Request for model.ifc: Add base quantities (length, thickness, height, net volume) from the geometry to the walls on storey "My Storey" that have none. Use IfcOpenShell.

First a look at what the model holds.

```python
import ifcopenshell
import ifcopenshell.util.element
import ifcopenshell.util.unit

model = ifcopenshell.open("model.ifc")
print(model.schema)
for unit_type in ("LENGTHUNIT", "AREAUNIT", "VOLUMEUNIT"):
    print(unit_type, ifcopenshell.util.unit.calculate_unit_scale(model, unit_type))
storey = next(s for s in model.by_type("IfcBuildingStorey") if s.Name == "My Storey")
walls = [e for e in ifcopenshell.util.element.get_decomposition(storey) if e.is_a("IfcWall")]
for e in sorted(walls, key=lambda e: e.id()):
    print(e.id(), e.is_a(), e.Name, list(ifcopenshell.util.element.get_psets(e, qtos_only=True)), sep=" | ")
```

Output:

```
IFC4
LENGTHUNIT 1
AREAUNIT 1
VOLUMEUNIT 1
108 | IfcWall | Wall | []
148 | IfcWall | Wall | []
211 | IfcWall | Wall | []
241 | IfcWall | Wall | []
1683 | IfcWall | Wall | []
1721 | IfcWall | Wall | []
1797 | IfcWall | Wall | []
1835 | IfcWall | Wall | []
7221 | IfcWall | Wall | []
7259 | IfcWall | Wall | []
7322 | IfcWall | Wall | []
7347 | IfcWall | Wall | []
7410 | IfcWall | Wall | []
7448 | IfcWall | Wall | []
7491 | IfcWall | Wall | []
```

```python
import ifcopenshell
import ifcopenshell.api.pset
import ifcopenshell.geom
import ifcopenshell.util.element
import ifcopenshell.util.shape
import ifcopenshell.util.unit

model = ifcopenshell.open("model.ifc")
unit_scale = ifcopenshell.util.unit.calculate_unit_scale(model)
volume_scale = ifcopenshell.util.unit.calculate_unit_scale(model, "VOLUMEUNIT")
settings = ifcopenshell.geom.settings()

storey = next(s for s in model.by_type("IfcBuildingStorey") if s.Name == "My Storey")
walls = [e for e in ifcopenshell.util.element.get_decomposition(storey) if e.is_a("IfcWall")]

for e in sorted(walls, key=lambda e: e.id()):
    if ifcopenshell.util.element.get_psets(e, qtos_only=True, should_inherit=False):
        continue
    # Geometry comes back in metres, in the element's own axes.
    shape = ifcopenshell.geom.create_shape(settings, e)
    values = {
        "Length": ifcopenshell.util.shape.get_x(shape.geometry) / unit_scale,
        "Width": ifcopenshell.util.shape.get_y(shape.geometry) / unit_scale,
        "Height": ifcopenshell.util.shape.get_z(shape.geometry) / unit_scale,
        "NetVolume": ifcopenshell.util.shape.get_volume(shape.geometry) / volume_scale,
    }
    qto = ifcopenshell.api.pset.add_qto(model, product=e, name="Qto_WallBaseQuantities")
    ifcopenshell.api.pset.edit_qto(model, qto=qto, properties=values)
    print(e.id(), {k: round(v, 3) for k, v in values.items()})

model.write("model_v2.ifc")
```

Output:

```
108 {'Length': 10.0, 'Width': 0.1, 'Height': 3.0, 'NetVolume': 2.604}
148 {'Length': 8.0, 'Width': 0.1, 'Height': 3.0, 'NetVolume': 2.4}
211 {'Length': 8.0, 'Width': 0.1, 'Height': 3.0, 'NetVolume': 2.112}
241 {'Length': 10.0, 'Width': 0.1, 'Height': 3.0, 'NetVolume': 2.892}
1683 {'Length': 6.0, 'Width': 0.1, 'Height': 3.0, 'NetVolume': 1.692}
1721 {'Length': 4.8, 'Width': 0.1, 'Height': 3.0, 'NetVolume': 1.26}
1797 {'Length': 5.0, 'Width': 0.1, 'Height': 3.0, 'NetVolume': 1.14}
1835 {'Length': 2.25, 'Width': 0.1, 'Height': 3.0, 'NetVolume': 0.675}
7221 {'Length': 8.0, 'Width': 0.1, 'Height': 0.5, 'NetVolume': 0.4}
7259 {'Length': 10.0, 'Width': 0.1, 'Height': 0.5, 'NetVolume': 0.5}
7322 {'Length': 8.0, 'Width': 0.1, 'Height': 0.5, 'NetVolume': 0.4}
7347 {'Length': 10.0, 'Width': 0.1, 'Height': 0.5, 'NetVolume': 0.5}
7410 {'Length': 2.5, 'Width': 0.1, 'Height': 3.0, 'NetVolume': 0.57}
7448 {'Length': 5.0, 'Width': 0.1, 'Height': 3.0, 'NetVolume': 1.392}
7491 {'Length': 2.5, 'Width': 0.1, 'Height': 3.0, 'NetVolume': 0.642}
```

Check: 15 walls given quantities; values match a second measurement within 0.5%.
